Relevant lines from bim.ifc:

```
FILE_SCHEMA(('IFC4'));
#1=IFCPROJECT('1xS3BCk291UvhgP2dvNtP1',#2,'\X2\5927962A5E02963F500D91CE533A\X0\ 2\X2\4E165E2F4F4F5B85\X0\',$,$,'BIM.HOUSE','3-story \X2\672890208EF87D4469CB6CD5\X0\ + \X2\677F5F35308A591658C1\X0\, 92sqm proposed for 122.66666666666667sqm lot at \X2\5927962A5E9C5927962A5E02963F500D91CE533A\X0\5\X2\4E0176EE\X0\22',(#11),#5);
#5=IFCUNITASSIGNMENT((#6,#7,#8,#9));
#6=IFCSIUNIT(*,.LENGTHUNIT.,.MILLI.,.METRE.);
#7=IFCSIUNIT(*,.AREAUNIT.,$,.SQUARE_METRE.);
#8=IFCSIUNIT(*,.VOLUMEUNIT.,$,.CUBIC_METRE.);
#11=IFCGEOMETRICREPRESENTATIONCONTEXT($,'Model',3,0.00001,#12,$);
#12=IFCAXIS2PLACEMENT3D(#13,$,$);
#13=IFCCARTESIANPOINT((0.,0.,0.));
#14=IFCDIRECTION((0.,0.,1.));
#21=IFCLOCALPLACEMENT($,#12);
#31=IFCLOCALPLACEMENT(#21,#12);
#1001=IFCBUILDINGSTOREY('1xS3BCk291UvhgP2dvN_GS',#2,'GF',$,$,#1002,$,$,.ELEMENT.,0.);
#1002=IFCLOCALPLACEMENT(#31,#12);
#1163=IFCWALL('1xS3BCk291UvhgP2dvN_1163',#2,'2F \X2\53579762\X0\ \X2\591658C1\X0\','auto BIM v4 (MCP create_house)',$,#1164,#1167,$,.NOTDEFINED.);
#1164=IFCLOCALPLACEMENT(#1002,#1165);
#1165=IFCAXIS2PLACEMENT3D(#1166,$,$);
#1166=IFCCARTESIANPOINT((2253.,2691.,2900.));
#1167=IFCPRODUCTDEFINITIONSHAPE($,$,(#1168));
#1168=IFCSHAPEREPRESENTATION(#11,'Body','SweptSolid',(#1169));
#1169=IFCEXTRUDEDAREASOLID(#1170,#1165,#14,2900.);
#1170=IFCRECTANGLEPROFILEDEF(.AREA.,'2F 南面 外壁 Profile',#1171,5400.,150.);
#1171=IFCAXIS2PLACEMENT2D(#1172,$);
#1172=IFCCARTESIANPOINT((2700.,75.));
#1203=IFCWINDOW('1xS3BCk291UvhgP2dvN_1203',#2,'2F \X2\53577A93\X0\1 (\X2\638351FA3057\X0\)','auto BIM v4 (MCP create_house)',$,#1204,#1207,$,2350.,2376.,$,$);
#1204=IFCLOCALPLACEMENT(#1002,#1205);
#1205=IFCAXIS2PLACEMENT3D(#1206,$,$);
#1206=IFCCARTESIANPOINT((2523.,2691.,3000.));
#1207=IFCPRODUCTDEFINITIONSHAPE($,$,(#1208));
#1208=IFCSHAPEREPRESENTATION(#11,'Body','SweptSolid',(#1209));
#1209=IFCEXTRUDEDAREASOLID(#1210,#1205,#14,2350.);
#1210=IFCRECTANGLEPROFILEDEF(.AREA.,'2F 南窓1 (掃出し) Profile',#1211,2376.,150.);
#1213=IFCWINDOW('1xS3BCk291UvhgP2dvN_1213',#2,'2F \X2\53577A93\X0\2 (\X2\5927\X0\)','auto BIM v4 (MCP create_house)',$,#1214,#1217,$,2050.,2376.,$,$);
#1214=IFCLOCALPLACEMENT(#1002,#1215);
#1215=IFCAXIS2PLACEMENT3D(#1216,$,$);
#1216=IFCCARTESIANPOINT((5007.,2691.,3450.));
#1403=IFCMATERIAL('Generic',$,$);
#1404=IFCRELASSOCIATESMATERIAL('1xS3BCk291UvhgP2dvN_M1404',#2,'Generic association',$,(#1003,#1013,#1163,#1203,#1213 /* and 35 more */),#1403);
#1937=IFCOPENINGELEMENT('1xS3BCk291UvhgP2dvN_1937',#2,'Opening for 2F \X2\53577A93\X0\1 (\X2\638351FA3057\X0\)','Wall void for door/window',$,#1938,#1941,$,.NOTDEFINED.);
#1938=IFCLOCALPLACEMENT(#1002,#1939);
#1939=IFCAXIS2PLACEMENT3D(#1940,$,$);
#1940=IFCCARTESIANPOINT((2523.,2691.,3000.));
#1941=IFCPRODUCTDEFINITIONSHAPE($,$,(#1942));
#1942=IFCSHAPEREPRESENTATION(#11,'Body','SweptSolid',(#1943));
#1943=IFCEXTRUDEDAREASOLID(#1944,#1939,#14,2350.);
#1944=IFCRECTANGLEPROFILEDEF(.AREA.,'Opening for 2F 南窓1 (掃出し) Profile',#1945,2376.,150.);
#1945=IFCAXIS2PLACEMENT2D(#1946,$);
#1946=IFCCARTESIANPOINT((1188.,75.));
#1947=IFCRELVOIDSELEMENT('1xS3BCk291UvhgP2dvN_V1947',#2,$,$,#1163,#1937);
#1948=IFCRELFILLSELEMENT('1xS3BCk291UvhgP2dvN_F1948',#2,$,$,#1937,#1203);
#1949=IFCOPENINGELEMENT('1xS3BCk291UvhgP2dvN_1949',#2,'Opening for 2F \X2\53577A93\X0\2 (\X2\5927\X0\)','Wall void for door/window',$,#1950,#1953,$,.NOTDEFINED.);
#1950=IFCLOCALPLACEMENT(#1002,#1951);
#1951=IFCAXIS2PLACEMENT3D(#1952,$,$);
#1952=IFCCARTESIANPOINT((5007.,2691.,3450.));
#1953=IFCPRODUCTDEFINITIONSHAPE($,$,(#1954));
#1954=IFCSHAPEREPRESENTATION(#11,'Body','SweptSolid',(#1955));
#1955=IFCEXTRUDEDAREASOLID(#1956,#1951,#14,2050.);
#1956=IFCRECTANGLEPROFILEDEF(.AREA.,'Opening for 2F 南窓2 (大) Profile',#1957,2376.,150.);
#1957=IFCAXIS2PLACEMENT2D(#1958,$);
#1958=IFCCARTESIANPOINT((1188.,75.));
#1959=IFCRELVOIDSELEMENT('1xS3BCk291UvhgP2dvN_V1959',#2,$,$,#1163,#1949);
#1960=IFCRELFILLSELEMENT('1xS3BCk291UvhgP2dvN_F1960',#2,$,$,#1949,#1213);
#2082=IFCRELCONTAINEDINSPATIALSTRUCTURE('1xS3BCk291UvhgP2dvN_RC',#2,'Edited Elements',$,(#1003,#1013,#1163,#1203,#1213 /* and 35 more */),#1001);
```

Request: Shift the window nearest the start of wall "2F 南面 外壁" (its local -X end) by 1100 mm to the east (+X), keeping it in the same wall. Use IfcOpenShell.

```python
import ifcopenshell
import ifcopenshell.api.geometry
import ifcopenshell.util.placement

model = ifcopenshell.open("bim.ifc")

window = model.by_guid("1xS3BCk291UvhgP2dvN_1203")
opening = window.FillsVoids[0].RelatingOpeningElement
wall = opening.VoidsElements[0].RelatingBuildingElement

wall_matrix = ifcopenshell.util.placement.get_local_placement(wall.ObjectPlacement)
shift = wall_matrix[:3, 0] * 1100.0
before = ifcopenshell.util.placement.get_local_placement(window.ObjectPlacement)[:3, 3].copy()

# The window is not placed relative to its opening, so move both.
for product in (opening, window):
    matrix = ifcopenshell.util.placement.get_local_placement(product.ObjectPlacement)
    matrix[:3, 3] += shift
    ifcopenshell.api.geometry.edit_object_placement(model, product=product, matrix=matrix, is_si=False)

after = ifcopenshell.util.placement.get_local_placement(window.ObjectPlacement)[:3, 3]
print("window moved by", (after - before).round(3) + 0.0)

model.write("bim_updated.ifc")
```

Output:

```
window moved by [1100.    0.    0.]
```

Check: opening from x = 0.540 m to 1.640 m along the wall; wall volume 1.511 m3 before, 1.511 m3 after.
